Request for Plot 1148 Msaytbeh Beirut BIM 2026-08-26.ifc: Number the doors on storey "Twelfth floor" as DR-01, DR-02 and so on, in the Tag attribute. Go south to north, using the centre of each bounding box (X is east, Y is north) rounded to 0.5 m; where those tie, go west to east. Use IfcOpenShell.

First a look at what the model holds.

```python
import ifcopenshell
import ifcopenshell.util.element
import ifcopenshell.util.placement

model = ifcopenshell.open("Plot 1148 Msaytbeh Beirut BIM 2026-08-26.ifc")
print(model.schema)
storey = next(s for s in model.by_type("IfcBuildingStorey") if s.Name == "Twelfth floor")
doors = [e for e in ifcopenshell.util.element.get_decomposition(storey) if e.is_a("IfcDoor")]
for e in sorted(doors, key=lambda e: e.id()):
    origin = ifcopenshell.util.placement.get_local_placement(e.ObjectPlacement)[:3, 3]
    print(e.id(), e.Tag, e.Name, origin.round(2) + 0.0, sep=" | ")
```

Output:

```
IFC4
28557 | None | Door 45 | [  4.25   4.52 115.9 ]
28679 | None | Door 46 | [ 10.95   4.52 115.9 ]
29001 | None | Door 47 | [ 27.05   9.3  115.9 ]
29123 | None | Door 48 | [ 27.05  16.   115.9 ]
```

```python
import ifcopenshell
import ifcopenshell.geom
import ifcopenshell.util.element
import ifcopenshell.util.shape

model = ifcopenshell.open("Plot 1148 Msaytbeh Beirut BIM 2026-08-26.ifc")
settings = ifcopenshell.geom.settings()
settings.set("use-world-coords", True)


def centre(element):
    shape = ifcopenshell.geom.create_shape(settings, element)
    return ifcopenshell.util.shape.get_bbox_centroid(shape.geometry)


storey = next(s for s in model.by_type("IfcBuildingStorey") if s.Name == "Twelfth floor")
doors = [e for e in ifcopenshell.util.element.get_decomposition(storey) if e.is_a("IfcDoor")]

# Insertion points can sit at a corner or the storey origin, so sort by the geometry (in metres).
centres = {e: centre(e) for e in doors}
doors.sort(key=lambda e: (round(centres[e][1] / 0.5), centres[e][0]))

for i, e in enumerate(doors, start=1):
    number = f"DR-{i:02d}"
    e.Tag = number
    print(e.id(), number)

model.write("Plot 1148 Msaytbeh Beirut BIM 2026-08-26_v2.ifc")
```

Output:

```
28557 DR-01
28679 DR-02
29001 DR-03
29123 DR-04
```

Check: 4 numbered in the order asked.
